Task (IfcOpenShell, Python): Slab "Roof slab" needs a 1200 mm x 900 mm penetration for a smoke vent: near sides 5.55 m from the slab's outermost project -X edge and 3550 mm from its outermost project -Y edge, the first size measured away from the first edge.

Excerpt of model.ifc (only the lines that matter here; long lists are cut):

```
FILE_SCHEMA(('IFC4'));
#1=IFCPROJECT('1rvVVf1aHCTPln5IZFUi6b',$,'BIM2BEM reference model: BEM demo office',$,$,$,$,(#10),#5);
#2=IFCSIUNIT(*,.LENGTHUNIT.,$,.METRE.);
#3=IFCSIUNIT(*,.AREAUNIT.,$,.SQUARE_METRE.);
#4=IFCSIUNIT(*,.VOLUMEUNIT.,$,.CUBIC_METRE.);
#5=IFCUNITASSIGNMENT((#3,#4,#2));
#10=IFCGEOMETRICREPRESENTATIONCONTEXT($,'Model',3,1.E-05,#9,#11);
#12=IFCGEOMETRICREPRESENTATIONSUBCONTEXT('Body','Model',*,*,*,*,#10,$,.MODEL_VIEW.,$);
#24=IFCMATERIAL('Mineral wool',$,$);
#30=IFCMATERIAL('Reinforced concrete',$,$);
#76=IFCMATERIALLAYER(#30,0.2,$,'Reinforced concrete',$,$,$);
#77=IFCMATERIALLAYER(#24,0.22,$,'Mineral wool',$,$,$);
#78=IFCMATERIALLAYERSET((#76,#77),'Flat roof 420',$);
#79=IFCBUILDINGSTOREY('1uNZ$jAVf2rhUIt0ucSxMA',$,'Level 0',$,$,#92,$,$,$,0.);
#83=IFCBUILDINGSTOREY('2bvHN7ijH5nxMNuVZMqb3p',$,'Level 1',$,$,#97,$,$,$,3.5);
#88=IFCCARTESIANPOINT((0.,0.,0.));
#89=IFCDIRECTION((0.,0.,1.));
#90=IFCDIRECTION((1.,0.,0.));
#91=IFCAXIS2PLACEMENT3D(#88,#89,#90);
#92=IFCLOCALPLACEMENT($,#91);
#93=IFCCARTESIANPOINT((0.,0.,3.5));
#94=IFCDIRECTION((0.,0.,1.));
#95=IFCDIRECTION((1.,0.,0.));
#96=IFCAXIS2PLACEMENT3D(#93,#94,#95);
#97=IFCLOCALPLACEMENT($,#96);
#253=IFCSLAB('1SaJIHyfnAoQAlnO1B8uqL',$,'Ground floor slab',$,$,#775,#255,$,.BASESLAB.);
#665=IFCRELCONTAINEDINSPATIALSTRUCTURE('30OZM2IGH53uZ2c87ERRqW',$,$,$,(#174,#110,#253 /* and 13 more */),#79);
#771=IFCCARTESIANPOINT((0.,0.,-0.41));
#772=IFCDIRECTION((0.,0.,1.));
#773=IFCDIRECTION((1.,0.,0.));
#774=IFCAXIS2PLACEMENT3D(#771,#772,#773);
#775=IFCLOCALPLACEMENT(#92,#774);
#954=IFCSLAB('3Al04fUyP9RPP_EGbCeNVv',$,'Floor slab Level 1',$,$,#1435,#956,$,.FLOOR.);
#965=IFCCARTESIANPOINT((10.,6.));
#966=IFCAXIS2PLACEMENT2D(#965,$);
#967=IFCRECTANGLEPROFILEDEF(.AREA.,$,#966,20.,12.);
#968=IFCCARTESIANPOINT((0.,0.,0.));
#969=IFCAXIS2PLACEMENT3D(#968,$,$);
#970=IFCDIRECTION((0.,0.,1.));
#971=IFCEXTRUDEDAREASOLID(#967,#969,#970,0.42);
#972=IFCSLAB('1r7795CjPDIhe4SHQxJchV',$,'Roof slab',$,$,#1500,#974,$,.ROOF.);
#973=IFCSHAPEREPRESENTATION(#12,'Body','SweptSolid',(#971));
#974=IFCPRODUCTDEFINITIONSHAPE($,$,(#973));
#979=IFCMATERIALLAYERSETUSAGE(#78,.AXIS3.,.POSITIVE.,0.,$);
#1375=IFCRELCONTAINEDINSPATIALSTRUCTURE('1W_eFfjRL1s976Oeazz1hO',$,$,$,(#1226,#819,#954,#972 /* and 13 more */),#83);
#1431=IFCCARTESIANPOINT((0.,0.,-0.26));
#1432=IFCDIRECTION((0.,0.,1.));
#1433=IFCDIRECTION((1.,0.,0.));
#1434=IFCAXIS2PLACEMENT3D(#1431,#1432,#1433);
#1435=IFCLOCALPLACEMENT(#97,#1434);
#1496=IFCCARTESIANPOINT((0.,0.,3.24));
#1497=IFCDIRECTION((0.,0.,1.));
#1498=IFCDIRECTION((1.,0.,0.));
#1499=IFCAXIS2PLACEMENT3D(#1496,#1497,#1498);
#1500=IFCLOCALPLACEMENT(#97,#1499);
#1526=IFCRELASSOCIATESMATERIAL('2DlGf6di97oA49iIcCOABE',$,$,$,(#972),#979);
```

```python
import numpy as np
import ifcopenshell
import ifcopenshell.api.feature
import ifcopenshell.api.geometry
import ifcopenshell.api.root
import ifcopenshell.geom
import ifcopenshell.util.placement
import ifcopenshell.util.representation
import ifcopenshell.util.shape
import ifcopenshell.util.unit

model = ifcopenshell.open("model.ifc")
unit_scale = ifcopenshell.util.unit.calculate_unit_scale(model)
settings = ifcopenshell.geom.settings()


def volume(element):
    """Net volume in cubic metres, openings subtracted."""
    shape = ifcopenshell.geom.create_shape(settings, element)
    return ifcopenshell.util.shape.get_volume(shape.geometry)


slab = model.by_guid("1r7795CjPDIhe4SHQxJchV")
before = volume(slab)

# Extent in the slab's own axes, in metres. The edges named are its -X and -Y sides.
slab_shape = ifcopenshell.geom.create_shape(settings, slab)
vertices = ifcopenshell.util.shape.get_vertices(slab_shape.geometry)
x_min, y_min, bottom = vertices.min(axis=0)
top = vertices[:, 2].max()

opening = ifcopenshell.api.root.create_entity(model, ifc_class="IfcOpeningElement", name="Smoke vent opening", predefined_type="OPENING")
context = ifcopenshell.util.representation.get_context(model, "Model", "Body", "MODEL_VIEW")
width, depth = 1.2, 0.9
outline = [(0.0, 0.0), (width, 0.0), (width, depth), (0.0, depth), (0.0, 0.0)]
# Overshoot both faces by 50 mm so the cut is clean.
shape = ifcopenshell.api.geometry.add_slab_representation(
    model, context=context, depth=top - bottom + 0.1, polyline=outline
)
ifcopenshell.api.geometry.assign_representation(model, product=opening, representation=shape)

matrix = ifcopenshell.util.placement.get_local_placement(slab.ObjectPlacement)
matrix[:, 3] = matrix @ np.append(np.array([x_min + 5.55, y_min + 3.55, bottom - 0.05]) / unit_scale, 1.0)
ifcopenshell.api.geometry.edit_object_placement(model, product=opening, matrix=matrix, is_si=False)
ifcopenshell.api.feature.add_feature(model, feature=opening, element=slab)

after = volume(slab)

print(f"slab volume {before:.3f} -> {after:.3f} m3")

model.write("model_edited.ifc")
```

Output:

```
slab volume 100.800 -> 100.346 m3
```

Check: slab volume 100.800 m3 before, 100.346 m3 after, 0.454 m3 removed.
